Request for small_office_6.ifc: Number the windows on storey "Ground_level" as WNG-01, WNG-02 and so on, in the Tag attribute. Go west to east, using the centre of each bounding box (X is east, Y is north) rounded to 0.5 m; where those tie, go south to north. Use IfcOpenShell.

First a look at what the model holds.

```python
import ifcopenshell
import ifcopenshell.util.element
import ifcopenshell.util.placement

model = ifcopenshell.open("small_office_6.ifc")
print(model.schema)
storey = next(s for s in model.by_type("IfcBuildingStorey") if s.Name == "Ground_level")
windows = [e for e in ifcopenshell.util.element.get_decomposition(storey) if e.is_a("IfcWindow")]
for e in sorted(windows, key=lambda e: e.id()):
    origin = ifcopenshell.util.placement.get_local_placement(e.ObjectPlacement)[:3, 3]
    print(e.id(), e.Tag, e.Name, origin.round(2) + 0.0, sep=" | ")
```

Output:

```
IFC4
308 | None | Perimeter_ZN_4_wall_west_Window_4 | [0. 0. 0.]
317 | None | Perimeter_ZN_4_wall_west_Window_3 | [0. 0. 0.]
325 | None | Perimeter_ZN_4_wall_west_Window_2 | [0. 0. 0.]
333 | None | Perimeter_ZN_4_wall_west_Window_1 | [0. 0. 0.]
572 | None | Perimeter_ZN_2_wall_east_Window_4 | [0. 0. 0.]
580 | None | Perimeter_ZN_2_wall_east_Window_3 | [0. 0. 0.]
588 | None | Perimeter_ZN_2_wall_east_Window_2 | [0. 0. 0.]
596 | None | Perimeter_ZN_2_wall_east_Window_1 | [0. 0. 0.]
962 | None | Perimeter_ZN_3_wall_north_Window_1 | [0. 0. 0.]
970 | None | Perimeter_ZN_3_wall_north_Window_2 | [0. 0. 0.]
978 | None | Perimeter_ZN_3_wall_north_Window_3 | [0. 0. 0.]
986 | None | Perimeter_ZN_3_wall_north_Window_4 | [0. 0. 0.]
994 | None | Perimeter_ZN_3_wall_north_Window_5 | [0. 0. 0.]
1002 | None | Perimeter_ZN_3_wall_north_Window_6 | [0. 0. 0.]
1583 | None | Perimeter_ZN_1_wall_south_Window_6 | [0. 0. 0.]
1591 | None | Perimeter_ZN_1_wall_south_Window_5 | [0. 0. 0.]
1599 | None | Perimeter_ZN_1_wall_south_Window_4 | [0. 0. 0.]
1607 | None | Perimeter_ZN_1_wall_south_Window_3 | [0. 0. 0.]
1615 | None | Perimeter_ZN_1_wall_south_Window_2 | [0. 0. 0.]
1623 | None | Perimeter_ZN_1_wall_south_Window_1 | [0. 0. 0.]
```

```python
import ifcopenshell
import ifcopenshell.geom
import ifcopenshell.util.element
import ifcopenshell.util.shape

model = ifcopenshell.open("small_office_6.ifc")
settings = ifcopenshell.geom.settings()
settings.set("use-world-coords", True)


def centre(element):
    shape = ifcopenshell.geom.create_shape(settings, element)
    return ifcopenshell.util.shape.get_bbox_centroid(shape.geometry)


storey = next(s for s in model.by_type("IfcBuildingStorey") if s.Name == "Ground_level")
windows = [e for e in ifcopenshell.util.element.get_decomposition(storey) if e.is_a("IfcWindow")]

# Insertion points can sit at a corner or the storey origin, so sort by the geometry (in metres).
centres = {e: centre(e) for e in windows}
windows.sort(key=lambda e: (round(centres[e][0] / 0.5), centres[e][1]))

for i, e in enumerate(windows, start=1):
    number = f"WNG-{i:02d}"
    e.Tag = number
    print(e.id(), number)

model.write("small_office_6_edited.ifc")
```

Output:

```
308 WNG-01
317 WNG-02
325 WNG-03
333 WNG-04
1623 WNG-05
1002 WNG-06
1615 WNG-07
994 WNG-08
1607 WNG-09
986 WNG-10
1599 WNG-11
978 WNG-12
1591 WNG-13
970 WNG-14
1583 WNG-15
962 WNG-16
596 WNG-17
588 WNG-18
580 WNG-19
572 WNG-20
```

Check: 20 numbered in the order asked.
